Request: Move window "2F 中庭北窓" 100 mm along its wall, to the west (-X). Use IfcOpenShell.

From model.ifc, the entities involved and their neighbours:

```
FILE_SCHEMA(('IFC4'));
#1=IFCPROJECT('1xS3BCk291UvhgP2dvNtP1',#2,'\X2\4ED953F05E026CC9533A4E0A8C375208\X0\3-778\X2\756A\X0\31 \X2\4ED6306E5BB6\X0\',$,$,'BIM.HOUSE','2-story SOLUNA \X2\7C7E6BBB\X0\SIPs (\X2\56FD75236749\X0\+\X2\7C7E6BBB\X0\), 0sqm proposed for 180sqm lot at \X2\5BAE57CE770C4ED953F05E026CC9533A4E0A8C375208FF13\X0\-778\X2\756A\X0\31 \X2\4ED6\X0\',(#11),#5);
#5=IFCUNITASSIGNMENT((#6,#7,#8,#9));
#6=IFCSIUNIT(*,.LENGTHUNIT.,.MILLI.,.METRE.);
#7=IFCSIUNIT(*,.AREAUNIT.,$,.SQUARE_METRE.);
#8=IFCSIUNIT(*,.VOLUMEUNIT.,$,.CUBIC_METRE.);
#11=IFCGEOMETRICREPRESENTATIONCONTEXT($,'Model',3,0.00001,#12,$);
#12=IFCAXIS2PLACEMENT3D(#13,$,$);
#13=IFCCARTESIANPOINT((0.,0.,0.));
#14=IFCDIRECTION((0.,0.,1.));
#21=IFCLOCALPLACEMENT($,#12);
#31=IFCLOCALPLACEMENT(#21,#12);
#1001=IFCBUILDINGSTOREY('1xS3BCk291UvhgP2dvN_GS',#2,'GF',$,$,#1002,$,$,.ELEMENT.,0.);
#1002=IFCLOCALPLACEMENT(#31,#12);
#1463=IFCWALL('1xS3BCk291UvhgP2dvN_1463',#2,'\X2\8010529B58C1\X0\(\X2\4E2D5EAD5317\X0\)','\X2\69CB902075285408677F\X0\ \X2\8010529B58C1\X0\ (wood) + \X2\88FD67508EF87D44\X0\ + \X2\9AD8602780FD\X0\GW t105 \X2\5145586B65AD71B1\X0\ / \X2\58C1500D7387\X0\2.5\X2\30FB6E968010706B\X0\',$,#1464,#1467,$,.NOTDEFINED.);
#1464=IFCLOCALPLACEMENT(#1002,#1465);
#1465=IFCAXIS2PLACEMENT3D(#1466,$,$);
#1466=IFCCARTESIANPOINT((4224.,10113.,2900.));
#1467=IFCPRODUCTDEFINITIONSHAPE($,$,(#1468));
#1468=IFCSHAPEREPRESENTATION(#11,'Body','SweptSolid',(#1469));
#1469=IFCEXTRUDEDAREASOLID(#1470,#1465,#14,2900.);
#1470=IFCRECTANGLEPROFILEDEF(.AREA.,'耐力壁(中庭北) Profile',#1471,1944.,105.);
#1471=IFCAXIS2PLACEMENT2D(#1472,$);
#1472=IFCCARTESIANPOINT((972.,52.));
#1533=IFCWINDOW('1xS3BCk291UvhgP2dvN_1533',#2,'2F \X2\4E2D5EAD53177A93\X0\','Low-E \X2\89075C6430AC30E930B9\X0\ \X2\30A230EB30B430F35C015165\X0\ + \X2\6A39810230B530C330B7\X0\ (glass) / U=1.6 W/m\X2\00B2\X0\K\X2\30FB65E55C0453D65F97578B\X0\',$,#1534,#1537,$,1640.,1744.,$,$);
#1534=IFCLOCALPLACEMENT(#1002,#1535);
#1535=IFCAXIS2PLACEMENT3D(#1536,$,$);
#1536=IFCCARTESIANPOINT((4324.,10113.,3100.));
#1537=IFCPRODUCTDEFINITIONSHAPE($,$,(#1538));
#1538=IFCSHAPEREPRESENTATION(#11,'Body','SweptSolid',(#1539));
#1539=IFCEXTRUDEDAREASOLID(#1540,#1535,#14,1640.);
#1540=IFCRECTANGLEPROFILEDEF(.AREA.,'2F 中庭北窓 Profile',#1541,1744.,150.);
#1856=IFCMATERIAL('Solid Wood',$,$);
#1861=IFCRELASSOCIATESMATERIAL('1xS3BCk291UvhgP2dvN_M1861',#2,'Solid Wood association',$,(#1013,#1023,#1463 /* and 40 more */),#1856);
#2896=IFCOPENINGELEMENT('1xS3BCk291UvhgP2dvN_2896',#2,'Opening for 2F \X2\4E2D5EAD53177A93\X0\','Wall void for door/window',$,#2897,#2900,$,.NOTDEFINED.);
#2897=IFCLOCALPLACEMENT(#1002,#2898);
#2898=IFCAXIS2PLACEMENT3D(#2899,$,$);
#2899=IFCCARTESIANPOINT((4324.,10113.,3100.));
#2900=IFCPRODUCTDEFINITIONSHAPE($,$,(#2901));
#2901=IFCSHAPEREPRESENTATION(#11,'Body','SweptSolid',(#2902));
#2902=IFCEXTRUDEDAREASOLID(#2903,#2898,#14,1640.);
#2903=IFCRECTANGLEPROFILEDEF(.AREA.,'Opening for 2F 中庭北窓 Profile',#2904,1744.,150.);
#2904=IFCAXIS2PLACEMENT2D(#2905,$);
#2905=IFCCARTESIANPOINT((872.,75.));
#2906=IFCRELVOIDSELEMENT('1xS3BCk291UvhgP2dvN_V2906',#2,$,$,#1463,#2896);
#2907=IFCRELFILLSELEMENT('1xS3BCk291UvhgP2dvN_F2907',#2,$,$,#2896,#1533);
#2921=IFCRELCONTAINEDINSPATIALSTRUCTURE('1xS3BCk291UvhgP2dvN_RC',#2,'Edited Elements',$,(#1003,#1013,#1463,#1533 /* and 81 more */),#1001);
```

```python
import ifcopenshell
import ifcopenshell.api.geometry
import ifcopenshell.util.placement

model = ifcopenshell.open("model.ifc")

window = model.by_guid("1xS3BCk291UvhgP2dvN_1533")
opening = window.FillsVoids[0].RelatingOpeningElement
wall = opening.VoidsElements[0].RelatingBuildingElement

wall_matrix = ifcopenshell.util.placement.get_local_placement(wall.ObjectPlacement)
shift = wall_matrix[:3, 0] * -100.0
before = ifcopenshell.util.placement.get_local_placement(window.ObjectPlacement)[:3, 3].copy()

# The window is not placed relative to its opening, so move both.
for product in (opening, window):
    matrix = ifcopenshell.util.placement.get_local_placement(product.ObjectPlacement)
    matrix[:3, 3] += shift
    ifcopenshell.api.geometry.edit_object_placement(model, product=product, matrix=matrix, is_si=False)

after = ifcopenshell.util.placement.get_local_placement(window.ObjectPlacement)[:3, 3]
print("window moved by", (after - before).round(3) + 0.0)

model.write("model_updated.ifc")
```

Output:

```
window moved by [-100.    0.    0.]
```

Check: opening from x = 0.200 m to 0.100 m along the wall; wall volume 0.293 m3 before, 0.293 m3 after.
